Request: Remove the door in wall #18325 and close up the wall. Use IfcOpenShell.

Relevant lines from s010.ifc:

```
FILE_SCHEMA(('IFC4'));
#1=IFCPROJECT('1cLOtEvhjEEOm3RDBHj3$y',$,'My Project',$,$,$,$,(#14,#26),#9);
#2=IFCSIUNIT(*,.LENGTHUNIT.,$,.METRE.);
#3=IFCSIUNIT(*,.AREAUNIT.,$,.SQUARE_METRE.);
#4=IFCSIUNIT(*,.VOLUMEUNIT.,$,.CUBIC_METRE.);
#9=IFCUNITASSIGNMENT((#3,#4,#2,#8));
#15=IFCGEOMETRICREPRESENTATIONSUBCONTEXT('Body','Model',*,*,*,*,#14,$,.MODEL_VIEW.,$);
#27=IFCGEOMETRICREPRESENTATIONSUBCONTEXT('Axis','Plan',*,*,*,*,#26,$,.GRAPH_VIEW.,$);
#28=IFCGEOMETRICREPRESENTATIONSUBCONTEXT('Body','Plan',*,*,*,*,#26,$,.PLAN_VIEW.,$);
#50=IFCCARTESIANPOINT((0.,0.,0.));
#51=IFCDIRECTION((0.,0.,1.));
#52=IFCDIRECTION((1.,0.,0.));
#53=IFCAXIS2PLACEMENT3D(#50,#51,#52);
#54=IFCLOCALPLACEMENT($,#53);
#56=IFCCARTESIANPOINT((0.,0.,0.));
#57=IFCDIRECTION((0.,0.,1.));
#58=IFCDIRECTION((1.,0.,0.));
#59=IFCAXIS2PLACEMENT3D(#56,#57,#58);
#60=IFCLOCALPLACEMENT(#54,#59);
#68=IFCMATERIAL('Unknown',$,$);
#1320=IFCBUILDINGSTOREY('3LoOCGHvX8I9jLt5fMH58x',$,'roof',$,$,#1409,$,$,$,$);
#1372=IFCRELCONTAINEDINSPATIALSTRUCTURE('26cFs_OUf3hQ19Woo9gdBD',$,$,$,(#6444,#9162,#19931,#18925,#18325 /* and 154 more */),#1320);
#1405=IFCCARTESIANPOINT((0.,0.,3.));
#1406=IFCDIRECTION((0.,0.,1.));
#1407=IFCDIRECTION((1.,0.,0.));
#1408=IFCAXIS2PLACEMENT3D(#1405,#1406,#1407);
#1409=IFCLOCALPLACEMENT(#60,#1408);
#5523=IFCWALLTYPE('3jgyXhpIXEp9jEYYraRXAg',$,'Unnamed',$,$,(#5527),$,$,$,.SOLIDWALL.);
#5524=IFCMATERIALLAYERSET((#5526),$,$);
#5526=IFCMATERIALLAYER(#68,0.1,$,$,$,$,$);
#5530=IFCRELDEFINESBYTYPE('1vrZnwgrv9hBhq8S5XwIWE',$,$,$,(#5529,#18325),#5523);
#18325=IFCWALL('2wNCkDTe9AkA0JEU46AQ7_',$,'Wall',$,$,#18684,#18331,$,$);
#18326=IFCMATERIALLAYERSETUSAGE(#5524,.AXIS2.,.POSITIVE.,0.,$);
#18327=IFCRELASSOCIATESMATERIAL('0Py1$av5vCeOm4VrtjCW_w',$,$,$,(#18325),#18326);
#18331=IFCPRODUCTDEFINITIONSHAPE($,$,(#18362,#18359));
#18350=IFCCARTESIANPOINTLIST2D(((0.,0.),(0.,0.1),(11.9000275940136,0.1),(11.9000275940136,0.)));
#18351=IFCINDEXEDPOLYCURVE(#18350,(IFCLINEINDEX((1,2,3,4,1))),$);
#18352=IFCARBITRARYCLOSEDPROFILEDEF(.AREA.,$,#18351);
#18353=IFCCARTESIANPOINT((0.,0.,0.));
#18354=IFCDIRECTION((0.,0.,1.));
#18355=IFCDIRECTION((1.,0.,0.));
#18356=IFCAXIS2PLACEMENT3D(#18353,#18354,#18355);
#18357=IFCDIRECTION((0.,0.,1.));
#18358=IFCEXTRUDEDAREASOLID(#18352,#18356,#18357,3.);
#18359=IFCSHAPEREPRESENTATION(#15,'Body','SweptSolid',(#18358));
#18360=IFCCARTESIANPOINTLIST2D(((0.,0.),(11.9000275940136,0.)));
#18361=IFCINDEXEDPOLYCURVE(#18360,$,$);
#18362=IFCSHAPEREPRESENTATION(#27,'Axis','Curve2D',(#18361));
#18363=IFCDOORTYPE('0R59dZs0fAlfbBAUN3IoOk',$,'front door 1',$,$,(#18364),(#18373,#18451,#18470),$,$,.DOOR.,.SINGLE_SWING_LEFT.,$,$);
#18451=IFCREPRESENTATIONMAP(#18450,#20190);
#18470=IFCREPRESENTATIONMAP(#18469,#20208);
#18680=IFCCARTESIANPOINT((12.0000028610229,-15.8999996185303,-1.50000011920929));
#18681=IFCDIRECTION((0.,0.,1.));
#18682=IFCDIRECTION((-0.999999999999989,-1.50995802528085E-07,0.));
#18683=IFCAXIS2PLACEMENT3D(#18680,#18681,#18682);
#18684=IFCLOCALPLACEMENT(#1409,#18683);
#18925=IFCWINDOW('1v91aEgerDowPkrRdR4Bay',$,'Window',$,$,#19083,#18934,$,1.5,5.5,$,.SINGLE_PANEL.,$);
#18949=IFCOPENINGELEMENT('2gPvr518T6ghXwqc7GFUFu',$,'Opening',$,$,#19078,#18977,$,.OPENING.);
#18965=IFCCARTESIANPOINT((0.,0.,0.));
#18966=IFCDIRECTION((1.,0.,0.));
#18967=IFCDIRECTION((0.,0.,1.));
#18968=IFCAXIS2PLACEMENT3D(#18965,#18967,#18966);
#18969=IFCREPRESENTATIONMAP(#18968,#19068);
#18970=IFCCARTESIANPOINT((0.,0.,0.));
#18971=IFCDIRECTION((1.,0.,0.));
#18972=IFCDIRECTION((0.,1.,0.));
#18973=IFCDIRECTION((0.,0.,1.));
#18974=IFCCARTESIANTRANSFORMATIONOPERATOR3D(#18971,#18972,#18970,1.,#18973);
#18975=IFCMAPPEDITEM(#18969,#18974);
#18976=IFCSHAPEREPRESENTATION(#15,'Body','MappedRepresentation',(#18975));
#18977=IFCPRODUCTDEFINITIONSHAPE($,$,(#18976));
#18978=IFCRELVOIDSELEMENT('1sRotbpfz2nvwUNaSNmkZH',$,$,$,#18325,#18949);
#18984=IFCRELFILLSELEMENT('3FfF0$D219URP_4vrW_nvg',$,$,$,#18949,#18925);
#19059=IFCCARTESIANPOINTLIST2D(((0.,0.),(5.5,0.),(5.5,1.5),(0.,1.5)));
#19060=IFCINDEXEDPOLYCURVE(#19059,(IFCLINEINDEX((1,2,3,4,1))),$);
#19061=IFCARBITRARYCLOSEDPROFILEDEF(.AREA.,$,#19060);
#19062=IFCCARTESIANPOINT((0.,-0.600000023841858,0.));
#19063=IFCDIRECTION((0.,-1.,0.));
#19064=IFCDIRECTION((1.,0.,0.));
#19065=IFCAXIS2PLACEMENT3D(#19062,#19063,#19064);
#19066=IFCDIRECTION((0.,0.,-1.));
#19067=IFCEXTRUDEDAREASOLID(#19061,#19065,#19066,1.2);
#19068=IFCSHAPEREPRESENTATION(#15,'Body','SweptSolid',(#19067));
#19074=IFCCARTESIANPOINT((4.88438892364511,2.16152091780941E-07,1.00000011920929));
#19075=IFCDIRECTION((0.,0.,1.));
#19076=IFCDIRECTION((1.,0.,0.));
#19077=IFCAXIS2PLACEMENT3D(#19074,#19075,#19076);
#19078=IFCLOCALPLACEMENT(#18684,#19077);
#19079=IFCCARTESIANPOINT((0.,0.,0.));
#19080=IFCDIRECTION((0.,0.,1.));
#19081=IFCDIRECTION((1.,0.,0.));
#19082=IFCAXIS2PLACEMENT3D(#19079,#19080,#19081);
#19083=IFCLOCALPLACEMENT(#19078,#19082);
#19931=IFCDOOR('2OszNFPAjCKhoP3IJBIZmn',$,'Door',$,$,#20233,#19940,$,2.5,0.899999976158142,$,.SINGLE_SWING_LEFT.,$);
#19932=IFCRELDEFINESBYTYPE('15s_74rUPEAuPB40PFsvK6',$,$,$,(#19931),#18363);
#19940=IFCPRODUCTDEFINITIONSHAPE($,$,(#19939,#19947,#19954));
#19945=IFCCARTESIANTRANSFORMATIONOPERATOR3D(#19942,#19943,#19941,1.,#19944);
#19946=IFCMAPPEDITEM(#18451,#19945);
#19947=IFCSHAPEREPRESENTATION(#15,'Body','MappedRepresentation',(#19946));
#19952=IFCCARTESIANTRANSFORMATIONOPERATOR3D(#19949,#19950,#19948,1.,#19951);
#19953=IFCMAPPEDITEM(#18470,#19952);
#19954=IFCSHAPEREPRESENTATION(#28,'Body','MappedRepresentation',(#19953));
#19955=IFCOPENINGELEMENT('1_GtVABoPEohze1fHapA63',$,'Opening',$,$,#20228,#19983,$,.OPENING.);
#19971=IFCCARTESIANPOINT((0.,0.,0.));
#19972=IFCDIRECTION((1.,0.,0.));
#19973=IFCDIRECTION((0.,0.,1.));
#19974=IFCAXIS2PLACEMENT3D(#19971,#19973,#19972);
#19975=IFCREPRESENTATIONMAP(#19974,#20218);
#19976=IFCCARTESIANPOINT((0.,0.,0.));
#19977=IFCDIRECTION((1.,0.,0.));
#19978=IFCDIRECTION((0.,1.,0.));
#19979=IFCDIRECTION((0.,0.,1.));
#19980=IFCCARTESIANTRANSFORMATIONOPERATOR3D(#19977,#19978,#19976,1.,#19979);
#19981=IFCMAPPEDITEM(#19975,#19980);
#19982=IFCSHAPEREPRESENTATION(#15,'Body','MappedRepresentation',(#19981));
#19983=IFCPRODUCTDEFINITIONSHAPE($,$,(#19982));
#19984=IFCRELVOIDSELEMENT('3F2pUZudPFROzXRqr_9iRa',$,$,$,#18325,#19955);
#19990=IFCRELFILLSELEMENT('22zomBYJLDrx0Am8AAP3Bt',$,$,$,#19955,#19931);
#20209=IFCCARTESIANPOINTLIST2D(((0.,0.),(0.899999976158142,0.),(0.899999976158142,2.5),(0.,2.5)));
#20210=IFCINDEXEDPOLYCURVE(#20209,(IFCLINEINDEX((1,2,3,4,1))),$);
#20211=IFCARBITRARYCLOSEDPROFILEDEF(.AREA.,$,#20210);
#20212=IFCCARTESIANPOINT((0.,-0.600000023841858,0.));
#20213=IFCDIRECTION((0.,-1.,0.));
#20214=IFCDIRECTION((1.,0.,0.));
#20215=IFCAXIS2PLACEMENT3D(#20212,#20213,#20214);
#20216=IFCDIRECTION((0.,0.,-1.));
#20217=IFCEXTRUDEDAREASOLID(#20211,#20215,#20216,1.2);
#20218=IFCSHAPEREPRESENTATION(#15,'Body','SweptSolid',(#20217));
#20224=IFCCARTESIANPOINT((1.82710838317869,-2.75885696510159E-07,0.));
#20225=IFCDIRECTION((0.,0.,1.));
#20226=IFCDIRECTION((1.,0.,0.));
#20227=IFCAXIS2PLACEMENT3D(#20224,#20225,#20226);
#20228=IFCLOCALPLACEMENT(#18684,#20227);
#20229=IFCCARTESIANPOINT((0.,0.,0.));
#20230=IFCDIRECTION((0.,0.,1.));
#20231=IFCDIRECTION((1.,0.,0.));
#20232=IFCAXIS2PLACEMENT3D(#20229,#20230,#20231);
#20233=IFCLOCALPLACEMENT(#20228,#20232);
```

```python
import ifcopenshell
import ifcopenshell.api.feature
import ifcopenshell.api.root
import ifcopenshell.geom
import ifcopenshell.util.shape

model = ifcopenshell.open("s010.ifc")
settings = ifcopenshell.geom.settings()


def volume(element):
    """Net volume in cubic metres, openings subtracted."""
    shape = ifcopenshell.geom.create_shape(settings, element)
    return ifcopenshell.util.shape.get_volume(shape.geometry)


door = model.by_id(19931)
opening = door.FillsVoids[0].RelatingOpeningElement
wall = opening.VoidsElements[0].RelatingBuildingElement
before = volume(wall)

ifcopenshell.api.root.remove_product(model, product=door)
ifcopenshell.api.feature.remove_feature(model, feature=opening)

after = volume(wall)

print(f"wall volume {before:.3f} -> {after:.3f} m3")

model.write("s010_v2.ifc")
```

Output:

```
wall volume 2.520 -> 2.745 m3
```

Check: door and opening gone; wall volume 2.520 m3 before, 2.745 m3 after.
